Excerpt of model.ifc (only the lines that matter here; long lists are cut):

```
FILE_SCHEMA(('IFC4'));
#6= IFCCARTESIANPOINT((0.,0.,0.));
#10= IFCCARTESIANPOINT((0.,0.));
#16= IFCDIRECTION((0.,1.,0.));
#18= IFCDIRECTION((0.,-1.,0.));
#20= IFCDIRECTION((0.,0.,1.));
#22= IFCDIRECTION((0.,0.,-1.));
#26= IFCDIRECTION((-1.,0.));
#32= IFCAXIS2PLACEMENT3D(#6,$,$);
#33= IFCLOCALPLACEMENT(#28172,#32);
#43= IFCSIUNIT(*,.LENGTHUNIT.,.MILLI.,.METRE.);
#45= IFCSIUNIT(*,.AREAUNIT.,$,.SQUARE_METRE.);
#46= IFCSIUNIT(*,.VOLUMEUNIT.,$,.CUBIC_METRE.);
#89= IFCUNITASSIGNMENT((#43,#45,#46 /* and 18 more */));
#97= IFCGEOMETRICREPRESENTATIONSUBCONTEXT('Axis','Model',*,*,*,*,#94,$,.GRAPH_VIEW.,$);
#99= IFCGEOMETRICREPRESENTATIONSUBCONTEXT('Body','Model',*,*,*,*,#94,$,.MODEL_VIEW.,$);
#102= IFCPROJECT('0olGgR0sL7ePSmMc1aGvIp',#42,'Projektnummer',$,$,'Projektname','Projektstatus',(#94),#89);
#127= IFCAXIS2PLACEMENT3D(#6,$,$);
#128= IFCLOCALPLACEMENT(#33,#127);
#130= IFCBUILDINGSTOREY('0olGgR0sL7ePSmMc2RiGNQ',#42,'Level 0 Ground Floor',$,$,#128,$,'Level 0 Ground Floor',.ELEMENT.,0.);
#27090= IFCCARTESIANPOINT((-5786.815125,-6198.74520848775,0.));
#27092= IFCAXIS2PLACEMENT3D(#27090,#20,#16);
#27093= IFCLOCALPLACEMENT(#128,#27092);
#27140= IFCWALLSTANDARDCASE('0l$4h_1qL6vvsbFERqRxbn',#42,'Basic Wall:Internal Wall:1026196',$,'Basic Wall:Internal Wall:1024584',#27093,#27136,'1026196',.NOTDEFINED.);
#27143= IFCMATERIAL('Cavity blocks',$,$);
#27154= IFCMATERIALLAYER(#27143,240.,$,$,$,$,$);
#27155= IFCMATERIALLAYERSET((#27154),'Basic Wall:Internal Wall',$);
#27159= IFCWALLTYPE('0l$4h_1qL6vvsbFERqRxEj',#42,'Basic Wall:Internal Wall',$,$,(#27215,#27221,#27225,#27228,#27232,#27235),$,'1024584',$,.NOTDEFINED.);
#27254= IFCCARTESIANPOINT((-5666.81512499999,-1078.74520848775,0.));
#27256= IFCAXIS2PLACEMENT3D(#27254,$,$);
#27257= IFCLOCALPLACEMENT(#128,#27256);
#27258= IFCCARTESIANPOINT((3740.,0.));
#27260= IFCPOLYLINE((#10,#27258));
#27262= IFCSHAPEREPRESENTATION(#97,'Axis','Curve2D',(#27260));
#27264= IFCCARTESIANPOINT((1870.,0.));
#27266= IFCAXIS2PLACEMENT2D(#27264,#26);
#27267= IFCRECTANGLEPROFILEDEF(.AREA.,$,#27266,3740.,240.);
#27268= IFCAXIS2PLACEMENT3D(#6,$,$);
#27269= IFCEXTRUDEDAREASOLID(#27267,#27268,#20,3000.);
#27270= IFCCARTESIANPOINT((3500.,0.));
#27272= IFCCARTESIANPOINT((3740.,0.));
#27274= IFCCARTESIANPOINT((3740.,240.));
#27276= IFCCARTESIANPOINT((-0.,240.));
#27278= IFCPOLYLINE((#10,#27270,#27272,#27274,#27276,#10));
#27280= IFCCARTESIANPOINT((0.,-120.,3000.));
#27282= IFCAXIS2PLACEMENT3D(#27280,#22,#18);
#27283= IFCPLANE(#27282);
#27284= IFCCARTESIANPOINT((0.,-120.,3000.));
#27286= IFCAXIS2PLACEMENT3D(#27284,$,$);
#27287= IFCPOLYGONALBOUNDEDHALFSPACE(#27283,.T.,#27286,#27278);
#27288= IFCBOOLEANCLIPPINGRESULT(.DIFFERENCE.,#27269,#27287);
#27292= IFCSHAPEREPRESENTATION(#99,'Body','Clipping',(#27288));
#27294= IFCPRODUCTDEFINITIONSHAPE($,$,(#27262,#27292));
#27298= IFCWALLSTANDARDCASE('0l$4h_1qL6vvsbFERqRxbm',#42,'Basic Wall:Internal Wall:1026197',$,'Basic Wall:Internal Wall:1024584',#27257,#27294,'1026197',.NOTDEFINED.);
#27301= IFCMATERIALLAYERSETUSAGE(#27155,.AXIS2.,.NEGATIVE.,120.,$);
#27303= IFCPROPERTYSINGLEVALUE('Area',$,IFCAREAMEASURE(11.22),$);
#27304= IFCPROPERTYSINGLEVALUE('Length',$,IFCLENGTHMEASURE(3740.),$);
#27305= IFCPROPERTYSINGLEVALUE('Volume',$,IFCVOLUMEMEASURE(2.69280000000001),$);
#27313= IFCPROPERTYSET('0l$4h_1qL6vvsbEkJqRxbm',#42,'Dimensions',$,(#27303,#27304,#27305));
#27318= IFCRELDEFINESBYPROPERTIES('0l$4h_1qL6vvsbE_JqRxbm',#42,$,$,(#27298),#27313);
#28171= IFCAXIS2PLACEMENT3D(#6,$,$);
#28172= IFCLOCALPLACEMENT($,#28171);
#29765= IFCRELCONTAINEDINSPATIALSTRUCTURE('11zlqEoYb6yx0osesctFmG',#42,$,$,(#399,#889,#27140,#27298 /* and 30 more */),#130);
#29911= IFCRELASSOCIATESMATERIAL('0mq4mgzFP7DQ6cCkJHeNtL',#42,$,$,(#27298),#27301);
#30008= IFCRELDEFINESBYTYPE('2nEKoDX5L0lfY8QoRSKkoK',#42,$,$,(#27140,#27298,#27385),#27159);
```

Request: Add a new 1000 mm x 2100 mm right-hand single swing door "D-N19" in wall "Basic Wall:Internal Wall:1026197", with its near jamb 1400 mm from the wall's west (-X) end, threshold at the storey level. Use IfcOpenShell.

```python
import numpy as np
import ifcopenshell
import ifcopenshell.api.feature
import ifcopenshell.api.geometry
import ifcopenshell.api.pset
import ifcopenshell.api.root
import ifcopenshell.api.spatial
import ifcopenshell.geom
import ifcopenshell.util.element
import ifcopenshell.util.placement
import ifcopenshell.util.representation
import ifcopenshell.util.shape
import ifcopenshell.util.unit

model = ifcopenshell.open("model.ifc")
unit_scale = ifcopenshell.util.unit.calculate_unit_scale(model)
area_scale = ifcopenshell.util.unit.calculate_unit_scale(model, "AREAUNIT")
volume_scale = ifcopenshell.util.unit.calculate_unit_scale(model, "VOLUMEUNIT")
settings = ifcopenshell.geom.settings()


def volume(element):
    """Net volume in cubic metres, openings subtracted."""
    shape = ifcopenshell.geom.create_shape(settings, element)
    return ifcopenshell.util.shape.get_volume(shape.geometry)


wall = model.by_guid("0l$4h_1qL6vvsbFERqRxbm")
storey = ifcopenshell.util.element.get_container(wall, ifc_class="IfcBuildingStorey")
context = ifcopenshell.util.representation.get_context(model, "Model", "Body", "MODEL_VIEW")
before = volume(wall)

width, height, from_end, sill = 1, 2.1, 1.4, 0.0  # metres

# The wall runs along its own X axis, and the end named is its -X end.
wall_shape = ifcopenshell.geom.create_shape(settings, wall)
x, y, z = ifcopenshell.util.shape.get_vertices(wall_shape.geometry).T
start = x.min() + from_end
face, thickness = float(y.min()), float(y.max() - y.min())
wall_matrix = ifcopenshell.util.placement.get_local_placement(wall.ObjectPlacement)
level = ifcopenshell.util.placement.get_local_placement(storey.ObjectPlacement)[2, 3]


def in_wall(x, y):
    """Placement at x, y metres in the wall's axes, at sill height."""
    matrix = wall_matrix.copy()
    matrix[:, 3] = wall_matrix @ np.array([x / unit_scale, y / unit_scale, 0.0, 1.0])
    matrix[2, 3] = level + sill / unit_scale
    return matrix


# Opening: a box that overshoots both wall faces by 50 mm.
opening = ifcopenshell.api.root.create_entity(model, ifc_class="IfcOpeningElement", predefined_type="OPENING")
box = ifcopenshell.api.geometry.add_wall_representation(
    model, context=context, length=width, height=height, thickness=thickness + 0.1
)
ifcopenshell.api.geometry.assign_representation(model, product=opening, representation=box)
ifcopenshell.api.geometry.edit_object_placement(model, product=opening, matrix=in_wall(start, face - 0.05), is_si=False)
ifcopenshell.api.feature.add_feature(model, feature=opening, element=wall)

door = ifcopenshell.api.root.create_entity(model, ifc_class="IfcDoor", name="D-N19", predefined_type="DOOR")
door.OverallWidth, door.OverallHeight = width / unit_scale, height / unit_scale
door.OperationType = "SINGLE_SWING_RIGHT"
body = ifcopenshell.api.geometry.add_door_representation(
    model,
    context=context,
    overall_width=door.OverallWidth,
    overall_height=door.OverallHeight,
    operation_type="SINGLE_SWING_RIGHT",
    lining_properties={"LiningDepth": thickness / unit_scale, "ThresholdDepth": thickness / unit_scale},
)
ifcopenshell.api.geometry.assign_representation(model, product=door, representation=body)
ifcopenshell.api.spatial.assign_container(model, products=[door], relating_structure=storey)
ifcopenshell.api.feature.add_filling(model, opening=opening, element=door)

# The lining spans the wall, so the door starts at the wall face.
ifcopenshell.api.geometry.edit_object_placement(model, product=door, matrix=in_wall(start, face), is_si=False)

after = volume(wall)

# Update the wall's stored quantities.
pset = model.by_id(ifcopenshell.util.element.get_pset(wall, "Dimensions", should_inherit=False)["id"])
ifcopenshell.api.pset.edit_pset(model, pset=pset, properties={
    "Area": model.create_entity("IfcAreaMeasure", after / thickness / area_scale),
    "Volume": model.create_entity("IfcVolumeMeasure", after / volume_scale),
})

print(f"wall volume {before:.3f} -> {after:.3f} m3")

model.write("model_updated.ifc")
```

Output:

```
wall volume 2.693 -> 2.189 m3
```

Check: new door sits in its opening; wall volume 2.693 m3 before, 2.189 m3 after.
